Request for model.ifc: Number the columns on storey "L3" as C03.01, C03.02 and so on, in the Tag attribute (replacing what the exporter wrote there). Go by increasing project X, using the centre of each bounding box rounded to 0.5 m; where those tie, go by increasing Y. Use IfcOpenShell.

First a look at what the model holds.

```python
import ifcopenshell
import ifcopenshell.util.element
import ifcopenshell.util.placement

model = ifcopenshell.open("model.ifc")
print(model.schema)
storey = next(s for s in model.by_type("IfcBuildingStorey") if s.Name == "L3")
columns = [e for e in ifcopenshell.util.element.get_decomposition(storey) if e.is_a("IfcColumn")]
for e in sorted(columns, key=lambda e: e.id()):
    origin = ifcopenshell.util.placement.get_local_placement(e.ObjectPlacement)[:3, 3]
    print(e.id(), e.Tag, e.Name, origin.round(2) + 0.0, sep=" | ")
```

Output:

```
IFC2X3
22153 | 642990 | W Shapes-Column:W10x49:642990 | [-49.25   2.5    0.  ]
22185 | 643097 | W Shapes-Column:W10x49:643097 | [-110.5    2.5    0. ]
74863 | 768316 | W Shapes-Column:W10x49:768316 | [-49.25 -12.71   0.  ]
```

```python
import ifcopenshell
import ifcopenshell.geom
import ifcopenshell.util.element
import ifcopenshell.util.shape

model = ifcopenshell.open("model.ifc")
settings = ifcopenshell.geom.settings()
settings.set("use-world-coords", True)


def centre(element):
    shape = ifcopenshell.geom.create_shape(settings, element)
    return ifcopenshell.util.shape.get_bbox_centroid(shape.geometry)


storey = next(s for s in model.by_type("IfcBuildingStorey") if s.Name == "L3")
columns = [e for e in ifcopenshell.util.element.get_decomposition(storey) if e.is_a("IfcColumn")]

# Insertion points can sit at a corner or the storey origin, so sort by the geometry (in metres).
centres = {e: centre(e) for e in columns}
columns.sort(key=lambda e: (round(centres[e][0] / 0.5), centres[e][1]))

for i, e in enumerate(columns, start=1):
    number = f"C03.{i:02d}"
    e.Tag = number
    print(e.id(), number)

model.write("model_edited.ifc")
```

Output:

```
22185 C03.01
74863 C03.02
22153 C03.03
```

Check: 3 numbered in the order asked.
